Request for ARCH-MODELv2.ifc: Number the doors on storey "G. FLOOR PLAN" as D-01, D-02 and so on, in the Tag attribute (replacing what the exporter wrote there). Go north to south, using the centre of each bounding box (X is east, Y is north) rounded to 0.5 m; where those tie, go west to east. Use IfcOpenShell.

First a look at what the model holds.

```python
import ifcopenshell
import ifcopenshell.util.element
import ifcopenshell.util.placement

model = ifcopenshell.open("ARCH-MODELv2.ifc")
print(model.schema)
storey = next(s for s in model.by_type("IfcBuildingStorey") if s.Name == "G. FLOOR PLAN")
doors = [e for e in ifcopenshell.util.element.get_decomposition(storey) if e.is_a("IfcDoor")]
for e in sorted(doors, key=lambda e: e.id()):
    origin = ifcopenshell.util.placement.get_local_placement(e.ObjectPlacement)[:3, 3]
    print(e.id(), e.Tag, e.Name, origin.round(2) + 0.0, sep=" | ")
```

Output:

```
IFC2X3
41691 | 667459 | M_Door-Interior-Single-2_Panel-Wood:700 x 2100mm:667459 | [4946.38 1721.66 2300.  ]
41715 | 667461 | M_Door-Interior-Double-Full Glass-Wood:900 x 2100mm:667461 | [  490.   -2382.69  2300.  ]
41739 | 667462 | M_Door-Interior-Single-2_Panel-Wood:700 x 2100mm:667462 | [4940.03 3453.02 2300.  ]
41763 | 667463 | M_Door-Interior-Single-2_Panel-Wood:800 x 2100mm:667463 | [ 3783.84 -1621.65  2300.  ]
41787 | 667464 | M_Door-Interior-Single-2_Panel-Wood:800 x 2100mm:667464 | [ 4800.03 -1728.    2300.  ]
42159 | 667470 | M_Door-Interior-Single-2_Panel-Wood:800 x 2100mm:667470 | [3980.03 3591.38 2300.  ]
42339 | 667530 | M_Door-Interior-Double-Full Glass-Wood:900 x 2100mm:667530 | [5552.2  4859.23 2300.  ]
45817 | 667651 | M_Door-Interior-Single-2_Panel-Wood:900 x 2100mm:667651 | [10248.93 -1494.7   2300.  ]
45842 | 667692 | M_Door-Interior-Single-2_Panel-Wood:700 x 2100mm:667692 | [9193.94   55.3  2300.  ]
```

```python
import ifcopenshell
import ifcopenshell.geom
import ifcopenshell.util.element
import ifcopenshell.util.shape

model = ifcopenshell.open("ARCH-MODELv2.ifc")
settings = ifcopenshell.geom.settings()
settings.set("use-world-coords", True)


def centre(element):
    shape = ifcopenshell.geom.create_shape(settings, element)
    return ifcopenshell.util.shape.get_bbox_centroid(shape.geometry)


storey = next(s for s in model.by_type("IfcBuildingStorey") if s.Name == "G. FLOOR PLAN")
doors = [e for e in ifcopenshell.util.element.get_decomposition(storey) if e.is_a("IfcDoor")]

# Insertion points can sit at a corner or the storey origin, so sort by the geometry (in metres).
centres = {e: centre(e) for e in doors}
doors.sort(key=lambda e: (-round(centres[e][1] / 0.5), centres[e][0]))

for i, e in enumerate(doors, start=1):
    number = f"D-{i:02d}"
    e.Tag = number
    print(e.id(), number)

model.write("ARCH-MODELv2_rev.ifc")
```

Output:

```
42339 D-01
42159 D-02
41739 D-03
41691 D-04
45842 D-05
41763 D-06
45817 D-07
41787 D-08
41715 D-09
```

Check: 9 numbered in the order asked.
